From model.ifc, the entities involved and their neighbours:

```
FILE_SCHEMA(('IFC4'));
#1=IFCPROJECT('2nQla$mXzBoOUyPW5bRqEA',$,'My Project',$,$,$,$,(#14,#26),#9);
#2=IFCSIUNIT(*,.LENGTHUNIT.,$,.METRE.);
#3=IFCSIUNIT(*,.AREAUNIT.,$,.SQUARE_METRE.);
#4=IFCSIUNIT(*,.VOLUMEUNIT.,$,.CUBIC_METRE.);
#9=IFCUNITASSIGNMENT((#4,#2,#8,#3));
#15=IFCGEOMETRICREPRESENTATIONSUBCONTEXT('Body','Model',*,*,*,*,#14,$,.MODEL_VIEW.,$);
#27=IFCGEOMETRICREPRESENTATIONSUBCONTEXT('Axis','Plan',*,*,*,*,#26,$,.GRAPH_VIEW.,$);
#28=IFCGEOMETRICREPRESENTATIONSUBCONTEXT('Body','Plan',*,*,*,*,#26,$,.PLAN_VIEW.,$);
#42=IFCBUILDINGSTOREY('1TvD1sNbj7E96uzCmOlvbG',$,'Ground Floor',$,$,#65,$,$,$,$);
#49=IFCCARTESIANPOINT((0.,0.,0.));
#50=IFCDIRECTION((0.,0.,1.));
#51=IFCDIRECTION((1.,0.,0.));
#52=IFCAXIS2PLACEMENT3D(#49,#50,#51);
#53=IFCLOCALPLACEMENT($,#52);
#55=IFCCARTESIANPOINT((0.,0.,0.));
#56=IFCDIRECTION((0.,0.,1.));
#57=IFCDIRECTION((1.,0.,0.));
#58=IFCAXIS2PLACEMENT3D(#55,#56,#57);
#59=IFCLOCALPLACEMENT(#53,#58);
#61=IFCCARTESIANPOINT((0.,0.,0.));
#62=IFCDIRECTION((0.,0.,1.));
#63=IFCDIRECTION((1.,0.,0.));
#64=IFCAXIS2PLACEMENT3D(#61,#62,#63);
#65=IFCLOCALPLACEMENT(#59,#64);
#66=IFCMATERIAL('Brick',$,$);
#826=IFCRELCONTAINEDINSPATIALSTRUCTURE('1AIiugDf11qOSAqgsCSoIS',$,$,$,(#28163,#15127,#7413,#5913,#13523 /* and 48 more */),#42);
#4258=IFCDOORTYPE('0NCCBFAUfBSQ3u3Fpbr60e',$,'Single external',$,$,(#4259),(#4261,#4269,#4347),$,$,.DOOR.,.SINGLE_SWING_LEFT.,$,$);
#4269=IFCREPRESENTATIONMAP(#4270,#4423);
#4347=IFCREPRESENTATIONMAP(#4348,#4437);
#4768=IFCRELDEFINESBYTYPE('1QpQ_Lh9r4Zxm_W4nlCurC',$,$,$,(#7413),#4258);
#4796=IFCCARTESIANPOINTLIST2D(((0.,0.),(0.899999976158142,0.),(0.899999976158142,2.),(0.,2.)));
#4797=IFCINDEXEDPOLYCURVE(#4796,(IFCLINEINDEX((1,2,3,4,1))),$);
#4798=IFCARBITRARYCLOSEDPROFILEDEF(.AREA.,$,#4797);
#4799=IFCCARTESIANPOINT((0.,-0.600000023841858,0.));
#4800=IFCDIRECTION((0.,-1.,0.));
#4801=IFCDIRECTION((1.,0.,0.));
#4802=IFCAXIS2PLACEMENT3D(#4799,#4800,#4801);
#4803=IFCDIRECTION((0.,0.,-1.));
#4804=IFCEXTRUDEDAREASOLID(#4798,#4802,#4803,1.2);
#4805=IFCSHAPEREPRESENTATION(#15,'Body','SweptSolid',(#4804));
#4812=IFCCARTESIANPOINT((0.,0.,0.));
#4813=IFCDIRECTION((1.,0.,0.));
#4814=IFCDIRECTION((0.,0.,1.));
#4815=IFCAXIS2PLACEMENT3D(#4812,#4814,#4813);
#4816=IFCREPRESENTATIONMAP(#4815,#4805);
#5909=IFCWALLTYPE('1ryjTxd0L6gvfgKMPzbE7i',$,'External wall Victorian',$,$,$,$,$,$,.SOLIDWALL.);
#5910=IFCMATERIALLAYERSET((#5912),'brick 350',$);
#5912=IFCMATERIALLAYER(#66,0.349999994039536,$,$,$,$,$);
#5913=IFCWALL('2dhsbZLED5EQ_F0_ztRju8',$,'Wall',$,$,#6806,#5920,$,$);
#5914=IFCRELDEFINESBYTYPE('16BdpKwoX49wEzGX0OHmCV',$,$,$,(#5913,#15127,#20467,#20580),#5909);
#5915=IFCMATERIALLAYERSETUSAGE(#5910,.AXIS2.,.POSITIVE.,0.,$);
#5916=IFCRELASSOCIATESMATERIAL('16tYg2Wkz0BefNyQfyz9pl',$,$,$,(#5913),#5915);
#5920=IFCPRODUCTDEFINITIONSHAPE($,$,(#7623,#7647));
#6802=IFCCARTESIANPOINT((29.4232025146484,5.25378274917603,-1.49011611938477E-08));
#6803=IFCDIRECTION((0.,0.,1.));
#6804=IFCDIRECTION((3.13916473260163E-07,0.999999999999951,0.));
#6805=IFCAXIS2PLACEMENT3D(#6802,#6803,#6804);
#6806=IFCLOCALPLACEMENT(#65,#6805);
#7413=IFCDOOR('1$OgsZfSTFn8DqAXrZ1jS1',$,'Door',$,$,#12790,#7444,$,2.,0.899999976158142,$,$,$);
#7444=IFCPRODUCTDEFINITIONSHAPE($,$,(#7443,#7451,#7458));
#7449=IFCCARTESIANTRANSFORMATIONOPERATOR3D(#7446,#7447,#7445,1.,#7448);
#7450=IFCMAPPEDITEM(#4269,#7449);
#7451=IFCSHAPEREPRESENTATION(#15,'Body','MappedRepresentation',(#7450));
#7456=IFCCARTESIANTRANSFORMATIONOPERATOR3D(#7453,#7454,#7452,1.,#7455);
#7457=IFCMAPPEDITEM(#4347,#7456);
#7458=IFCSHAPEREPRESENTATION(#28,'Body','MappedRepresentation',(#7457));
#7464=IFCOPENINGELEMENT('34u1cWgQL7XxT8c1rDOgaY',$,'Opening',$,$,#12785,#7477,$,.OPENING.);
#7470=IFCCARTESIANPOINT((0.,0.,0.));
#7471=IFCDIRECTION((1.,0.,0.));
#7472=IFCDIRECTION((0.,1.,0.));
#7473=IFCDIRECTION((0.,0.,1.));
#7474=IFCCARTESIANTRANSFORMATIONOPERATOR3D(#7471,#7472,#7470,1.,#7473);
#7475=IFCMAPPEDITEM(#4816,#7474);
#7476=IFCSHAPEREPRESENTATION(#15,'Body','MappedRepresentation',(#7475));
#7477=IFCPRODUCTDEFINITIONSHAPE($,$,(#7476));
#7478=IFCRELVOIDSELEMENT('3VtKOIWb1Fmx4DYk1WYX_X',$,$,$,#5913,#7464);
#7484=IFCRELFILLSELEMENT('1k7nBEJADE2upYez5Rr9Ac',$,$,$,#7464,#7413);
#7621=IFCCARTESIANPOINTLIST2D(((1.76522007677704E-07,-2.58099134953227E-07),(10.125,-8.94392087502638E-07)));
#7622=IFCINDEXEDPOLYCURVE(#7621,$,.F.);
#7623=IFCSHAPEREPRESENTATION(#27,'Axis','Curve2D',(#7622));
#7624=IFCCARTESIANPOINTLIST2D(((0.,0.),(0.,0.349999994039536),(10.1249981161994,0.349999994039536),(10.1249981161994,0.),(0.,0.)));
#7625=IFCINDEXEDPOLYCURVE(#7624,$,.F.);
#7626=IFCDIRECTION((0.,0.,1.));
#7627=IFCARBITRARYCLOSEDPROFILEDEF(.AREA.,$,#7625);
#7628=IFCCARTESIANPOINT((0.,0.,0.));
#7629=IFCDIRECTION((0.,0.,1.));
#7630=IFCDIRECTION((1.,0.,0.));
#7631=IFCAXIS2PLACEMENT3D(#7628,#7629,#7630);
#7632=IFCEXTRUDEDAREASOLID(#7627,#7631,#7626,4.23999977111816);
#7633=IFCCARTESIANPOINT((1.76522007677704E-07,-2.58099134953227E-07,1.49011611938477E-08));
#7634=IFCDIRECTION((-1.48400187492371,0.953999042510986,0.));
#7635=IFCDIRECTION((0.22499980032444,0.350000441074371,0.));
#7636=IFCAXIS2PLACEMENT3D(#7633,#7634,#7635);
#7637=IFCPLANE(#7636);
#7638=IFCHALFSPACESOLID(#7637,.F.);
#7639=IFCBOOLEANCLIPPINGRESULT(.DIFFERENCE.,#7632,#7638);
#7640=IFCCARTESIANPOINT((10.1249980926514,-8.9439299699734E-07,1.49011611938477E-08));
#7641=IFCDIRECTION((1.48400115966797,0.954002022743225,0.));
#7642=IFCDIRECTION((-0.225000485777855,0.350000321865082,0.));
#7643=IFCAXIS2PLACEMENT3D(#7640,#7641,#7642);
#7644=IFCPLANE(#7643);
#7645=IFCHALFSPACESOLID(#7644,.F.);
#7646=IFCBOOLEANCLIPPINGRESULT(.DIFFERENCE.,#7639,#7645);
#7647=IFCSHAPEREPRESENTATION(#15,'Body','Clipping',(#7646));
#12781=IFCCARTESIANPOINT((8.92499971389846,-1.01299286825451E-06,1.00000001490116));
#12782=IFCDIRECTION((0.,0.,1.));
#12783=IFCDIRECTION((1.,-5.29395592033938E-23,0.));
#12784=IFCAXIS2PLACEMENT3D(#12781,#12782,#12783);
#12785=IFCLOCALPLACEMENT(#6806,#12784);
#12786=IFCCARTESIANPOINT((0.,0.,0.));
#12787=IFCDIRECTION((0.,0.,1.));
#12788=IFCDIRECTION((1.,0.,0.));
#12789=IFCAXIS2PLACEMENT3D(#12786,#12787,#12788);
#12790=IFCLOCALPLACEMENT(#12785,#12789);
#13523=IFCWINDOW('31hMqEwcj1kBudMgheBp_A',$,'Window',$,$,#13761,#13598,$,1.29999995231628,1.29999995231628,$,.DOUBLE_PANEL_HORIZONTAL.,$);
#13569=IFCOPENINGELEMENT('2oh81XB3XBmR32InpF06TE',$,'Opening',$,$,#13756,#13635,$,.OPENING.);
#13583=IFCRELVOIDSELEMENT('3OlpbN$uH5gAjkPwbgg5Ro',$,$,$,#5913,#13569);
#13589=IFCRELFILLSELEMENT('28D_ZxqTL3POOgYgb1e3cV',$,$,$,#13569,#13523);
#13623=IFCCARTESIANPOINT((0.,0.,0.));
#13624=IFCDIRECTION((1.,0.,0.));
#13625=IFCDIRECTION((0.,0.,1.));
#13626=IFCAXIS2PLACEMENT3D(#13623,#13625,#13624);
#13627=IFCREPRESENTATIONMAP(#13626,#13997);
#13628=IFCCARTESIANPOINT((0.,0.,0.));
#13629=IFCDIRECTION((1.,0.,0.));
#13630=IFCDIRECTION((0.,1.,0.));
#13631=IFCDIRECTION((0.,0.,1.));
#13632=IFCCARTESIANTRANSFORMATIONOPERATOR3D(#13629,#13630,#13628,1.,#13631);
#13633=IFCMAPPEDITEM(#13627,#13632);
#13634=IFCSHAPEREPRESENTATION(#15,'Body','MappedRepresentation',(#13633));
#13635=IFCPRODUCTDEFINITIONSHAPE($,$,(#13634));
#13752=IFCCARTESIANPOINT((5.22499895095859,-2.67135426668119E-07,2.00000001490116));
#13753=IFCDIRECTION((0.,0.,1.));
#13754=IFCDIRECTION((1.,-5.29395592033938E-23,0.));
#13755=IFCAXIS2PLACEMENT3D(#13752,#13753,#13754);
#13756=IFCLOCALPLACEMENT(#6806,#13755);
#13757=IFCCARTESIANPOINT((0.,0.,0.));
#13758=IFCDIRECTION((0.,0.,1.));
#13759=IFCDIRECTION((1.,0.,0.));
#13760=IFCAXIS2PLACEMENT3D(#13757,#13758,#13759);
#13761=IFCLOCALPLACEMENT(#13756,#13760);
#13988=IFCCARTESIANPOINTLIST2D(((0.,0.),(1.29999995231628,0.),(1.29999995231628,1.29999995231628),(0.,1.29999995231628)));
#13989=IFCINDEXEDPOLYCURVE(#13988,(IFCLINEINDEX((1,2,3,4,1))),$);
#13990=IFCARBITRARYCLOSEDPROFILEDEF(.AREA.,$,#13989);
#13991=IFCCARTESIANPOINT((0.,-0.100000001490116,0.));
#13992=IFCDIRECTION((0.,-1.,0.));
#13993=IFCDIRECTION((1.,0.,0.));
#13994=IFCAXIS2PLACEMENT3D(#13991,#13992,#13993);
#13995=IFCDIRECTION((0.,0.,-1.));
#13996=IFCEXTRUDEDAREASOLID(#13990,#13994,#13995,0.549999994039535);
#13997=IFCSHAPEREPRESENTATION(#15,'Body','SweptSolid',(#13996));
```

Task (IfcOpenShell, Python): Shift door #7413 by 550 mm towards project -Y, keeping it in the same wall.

```python
import ifcopenshell
import ifcopenshell.api.geometry
import ifcopenshell.util.placement
import ifcopenshell.util.unit

model = ifcopenshell.open("model.ifc")
unit_scale = ifcopenshell.util.unit.calculate_unit_scale(model)

door = model.by_guid("1$OgsZfSTFn8DqAXrZ1jS1")
opening = door.FillsVoids[0].RelatingOpeningElement
wall = opening.VoidsElements[0].RelatingBuildingElement

wall_matrix = ifcopenshell.util.placement.get_local_placement(wall.ObjectPlacement)
shift = wall_matrix[:3, 0] * -0.55 / unit_scale
before = ifcopenshell.util.placement.get_local_placement(door.ObjectPlacement)[:3, 3].copy()

# The door is placed relative to its opening, so it follows when the opening moves.
matrix = ifcopenshell.util.placement.get_local_placement(opening.ObjectPlacement)
matrix[:3, 3] += shift
ifcopenshell.api.geometry.edit_object_placement(
    model, product=opening, matrix=matrix, is_si=False, should_transform_children=True
)

after = ifcopenshell.util.placement.get_local_placement(door.ObjectPlacement)[:3, 3]
print("door moved by", (after - before).round(3) + 0.0)

model.write("model_v2.ifc")
```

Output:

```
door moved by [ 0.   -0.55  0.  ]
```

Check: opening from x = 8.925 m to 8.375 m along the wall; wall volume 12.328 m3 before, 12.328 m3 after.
